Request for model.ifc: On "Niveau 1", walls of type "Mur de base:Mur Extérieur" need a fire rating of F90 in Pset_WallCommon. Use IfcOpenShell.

First a look at what the model holds.

```python
import ifcopenshell
import ifcopenshell.util.element

model = ifcopenshell.open("model.ifc")
print(model.schema)
storey = next(s for s in model.by_type("IfcBuildingStorey") if s.Name == "Niveau 1")
walls = [e for e in ifcopenshell.util.element.get_decomposition(storey) if e.is_a("IfcWall")]
seen = {}
for e in walls:
    element_type = ifcopenshell.util.element.get_type(e)
    key = (element_type.Name if element_type != e and element_type else None, ifcopenshell.util.element.get_pset(e, "Pset_WallCommon", "FireRating"))
    seen[key] = seen.get(key, 0) + 1
for (name, value), count in sorted(seen.items(), key=str):
    print(count, "x", name, "|", value)
```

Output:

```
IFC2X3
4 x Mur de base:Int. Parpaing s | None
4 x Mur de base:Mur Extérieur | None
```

```python
import ifcopenshell
import ifcopenshell.api.pset
import ifcopenshell.util.element

model = ifcopenshell.open("model.ifc")

storey = next(s for s in model.by_type("IfcBuildingStorey") if s.Name == "Niveau 1")
walls = [e for e in ifcopenshell.util.element.get_decomposition(storey) if e.is_a("IfcWall")]

count = 0
for e in walls:
    element_type = ifcopenshell.util.element.get_type(e)
    if element_type in (None, e) or element_type.Name != "Mur de base:Mur Extérieur":
        continue
    # add_pset returns the element's existing set when there is one.
    pset = ifcopenshell.api.pset.add_pset(model, product=e, name="Pset_WallCommon")
    ifcopenshell.api.pset.edit_pset(model, pset=pset, properties={"FireRating": "F90"})
    count += 1

print(count, "walls updated")

model.write("model_updated.ifc")
```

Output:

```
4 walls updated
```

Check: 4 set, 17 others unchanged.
